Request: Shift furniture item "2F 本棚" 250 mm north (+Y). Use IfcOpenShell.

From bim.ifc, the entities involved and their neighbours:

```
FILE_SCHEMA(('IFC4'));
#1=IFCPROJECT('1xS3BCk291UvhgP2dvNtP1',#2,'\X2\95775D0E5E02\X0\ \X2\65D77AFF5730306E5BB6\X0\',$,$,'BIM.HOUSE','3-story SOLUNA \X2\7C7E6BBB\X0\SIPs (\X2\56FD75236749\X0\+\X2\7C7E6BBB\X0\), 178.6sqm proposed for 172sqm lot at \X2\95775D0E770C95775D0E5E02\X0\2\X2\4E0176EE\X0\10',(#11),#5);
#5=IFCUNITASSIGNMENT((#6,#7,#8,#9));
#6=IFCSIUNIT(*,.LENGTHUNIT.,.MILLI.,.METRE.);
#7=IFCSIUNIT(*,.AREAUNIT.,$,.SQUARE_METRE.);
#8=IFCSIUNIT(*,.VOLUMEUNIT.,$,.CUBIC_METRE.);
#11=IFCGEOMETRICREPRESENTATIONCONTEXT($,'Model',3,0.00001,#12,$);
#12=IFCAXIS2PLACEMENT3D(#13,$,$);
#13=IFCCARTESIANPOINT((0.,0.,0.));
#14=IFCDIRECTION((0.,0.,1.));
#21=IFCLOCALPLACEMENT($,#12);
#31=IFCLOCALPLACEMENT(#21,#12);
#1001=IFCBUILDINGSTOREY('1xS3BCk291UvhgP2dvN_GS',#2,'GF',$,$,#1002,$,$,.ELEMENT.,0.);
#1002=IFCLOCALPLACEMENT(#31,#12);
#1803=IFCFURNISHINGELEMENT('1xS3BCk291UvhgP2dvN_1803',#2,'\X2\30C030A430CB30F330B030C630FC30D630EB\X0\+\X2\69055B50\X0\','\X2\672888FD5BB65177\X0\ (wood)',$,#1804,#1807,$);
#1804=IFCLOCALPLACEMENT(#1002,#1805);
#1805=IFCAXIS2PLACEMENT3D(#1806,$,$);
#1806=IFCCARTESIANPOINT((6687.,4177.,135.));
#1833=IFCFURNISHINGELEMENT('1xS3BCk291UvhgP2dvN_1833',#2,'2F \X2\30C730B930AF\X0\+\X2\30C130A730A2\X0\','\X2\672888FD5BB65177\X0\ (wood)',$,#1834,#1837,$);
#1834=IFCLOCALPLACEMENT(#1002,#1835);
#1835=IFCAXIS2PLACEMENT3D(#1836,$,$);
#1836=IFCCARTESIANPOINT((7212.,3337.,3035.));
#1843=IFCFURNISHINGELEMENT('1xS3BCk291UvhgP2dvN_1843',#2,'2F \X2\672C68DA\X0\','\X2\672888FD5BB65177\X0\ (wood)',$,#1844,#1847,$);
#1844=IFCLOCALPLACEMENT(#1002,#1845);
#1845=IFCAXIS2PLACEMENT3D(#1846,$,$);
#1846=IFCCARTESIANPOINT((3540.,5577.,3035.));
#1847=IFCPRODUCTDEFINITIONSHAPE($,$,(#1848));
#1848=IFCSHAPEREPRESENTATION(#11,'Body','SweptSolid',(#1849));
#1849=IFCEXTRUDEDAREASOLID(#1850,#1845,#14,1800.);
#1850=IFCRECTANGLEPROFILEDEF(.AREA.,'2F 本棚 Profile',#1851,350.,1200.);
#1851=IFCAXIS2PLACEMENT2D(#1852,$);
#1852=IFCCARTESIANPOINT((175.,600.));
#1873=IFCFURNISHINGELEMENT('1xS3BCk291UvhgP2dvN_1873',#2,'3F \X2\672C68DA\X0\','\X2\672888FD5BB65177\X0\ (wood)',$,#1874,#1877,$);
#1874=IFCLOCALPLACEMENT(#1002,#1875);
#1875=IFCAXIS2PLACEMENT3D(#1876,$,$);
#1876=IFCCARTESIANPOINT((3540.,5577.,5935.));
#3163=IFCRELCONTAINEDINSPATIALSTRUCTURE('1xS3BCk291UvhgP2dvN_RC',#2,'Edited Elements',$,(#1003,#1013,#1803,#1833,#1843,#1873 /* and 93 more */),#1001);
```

```python
import ifcopenshell
import ifcopenshell.api.geometry
import ifcopenshell.util.placement

model = ifcopenshell.open("bim.ifc")

item = model.by_guid("1xS3BCk291UvhgP2dvN_1843")
matrix = ifcopenshell.util.placement.get_local_placement(item.ObjectPlacement)
matrix[1, 3] += 250.0
ifcopenshell.api.geometry.edit_object_placement(model, product=item, matrix=matrix, is_si=False)

print(ifcopenshell.util.placement.get_local_placement(item.ObjectPlacement).round(3) + 0.0)

model.write("bim_v2.ifc")
```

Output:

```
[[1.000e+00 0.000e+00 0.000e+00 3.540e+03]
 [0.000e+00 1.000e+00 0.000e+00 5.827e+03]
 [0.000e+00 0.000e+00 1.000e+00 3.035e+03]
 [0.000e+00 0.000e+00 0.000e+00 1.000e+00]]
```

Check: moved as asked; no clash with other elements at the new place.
